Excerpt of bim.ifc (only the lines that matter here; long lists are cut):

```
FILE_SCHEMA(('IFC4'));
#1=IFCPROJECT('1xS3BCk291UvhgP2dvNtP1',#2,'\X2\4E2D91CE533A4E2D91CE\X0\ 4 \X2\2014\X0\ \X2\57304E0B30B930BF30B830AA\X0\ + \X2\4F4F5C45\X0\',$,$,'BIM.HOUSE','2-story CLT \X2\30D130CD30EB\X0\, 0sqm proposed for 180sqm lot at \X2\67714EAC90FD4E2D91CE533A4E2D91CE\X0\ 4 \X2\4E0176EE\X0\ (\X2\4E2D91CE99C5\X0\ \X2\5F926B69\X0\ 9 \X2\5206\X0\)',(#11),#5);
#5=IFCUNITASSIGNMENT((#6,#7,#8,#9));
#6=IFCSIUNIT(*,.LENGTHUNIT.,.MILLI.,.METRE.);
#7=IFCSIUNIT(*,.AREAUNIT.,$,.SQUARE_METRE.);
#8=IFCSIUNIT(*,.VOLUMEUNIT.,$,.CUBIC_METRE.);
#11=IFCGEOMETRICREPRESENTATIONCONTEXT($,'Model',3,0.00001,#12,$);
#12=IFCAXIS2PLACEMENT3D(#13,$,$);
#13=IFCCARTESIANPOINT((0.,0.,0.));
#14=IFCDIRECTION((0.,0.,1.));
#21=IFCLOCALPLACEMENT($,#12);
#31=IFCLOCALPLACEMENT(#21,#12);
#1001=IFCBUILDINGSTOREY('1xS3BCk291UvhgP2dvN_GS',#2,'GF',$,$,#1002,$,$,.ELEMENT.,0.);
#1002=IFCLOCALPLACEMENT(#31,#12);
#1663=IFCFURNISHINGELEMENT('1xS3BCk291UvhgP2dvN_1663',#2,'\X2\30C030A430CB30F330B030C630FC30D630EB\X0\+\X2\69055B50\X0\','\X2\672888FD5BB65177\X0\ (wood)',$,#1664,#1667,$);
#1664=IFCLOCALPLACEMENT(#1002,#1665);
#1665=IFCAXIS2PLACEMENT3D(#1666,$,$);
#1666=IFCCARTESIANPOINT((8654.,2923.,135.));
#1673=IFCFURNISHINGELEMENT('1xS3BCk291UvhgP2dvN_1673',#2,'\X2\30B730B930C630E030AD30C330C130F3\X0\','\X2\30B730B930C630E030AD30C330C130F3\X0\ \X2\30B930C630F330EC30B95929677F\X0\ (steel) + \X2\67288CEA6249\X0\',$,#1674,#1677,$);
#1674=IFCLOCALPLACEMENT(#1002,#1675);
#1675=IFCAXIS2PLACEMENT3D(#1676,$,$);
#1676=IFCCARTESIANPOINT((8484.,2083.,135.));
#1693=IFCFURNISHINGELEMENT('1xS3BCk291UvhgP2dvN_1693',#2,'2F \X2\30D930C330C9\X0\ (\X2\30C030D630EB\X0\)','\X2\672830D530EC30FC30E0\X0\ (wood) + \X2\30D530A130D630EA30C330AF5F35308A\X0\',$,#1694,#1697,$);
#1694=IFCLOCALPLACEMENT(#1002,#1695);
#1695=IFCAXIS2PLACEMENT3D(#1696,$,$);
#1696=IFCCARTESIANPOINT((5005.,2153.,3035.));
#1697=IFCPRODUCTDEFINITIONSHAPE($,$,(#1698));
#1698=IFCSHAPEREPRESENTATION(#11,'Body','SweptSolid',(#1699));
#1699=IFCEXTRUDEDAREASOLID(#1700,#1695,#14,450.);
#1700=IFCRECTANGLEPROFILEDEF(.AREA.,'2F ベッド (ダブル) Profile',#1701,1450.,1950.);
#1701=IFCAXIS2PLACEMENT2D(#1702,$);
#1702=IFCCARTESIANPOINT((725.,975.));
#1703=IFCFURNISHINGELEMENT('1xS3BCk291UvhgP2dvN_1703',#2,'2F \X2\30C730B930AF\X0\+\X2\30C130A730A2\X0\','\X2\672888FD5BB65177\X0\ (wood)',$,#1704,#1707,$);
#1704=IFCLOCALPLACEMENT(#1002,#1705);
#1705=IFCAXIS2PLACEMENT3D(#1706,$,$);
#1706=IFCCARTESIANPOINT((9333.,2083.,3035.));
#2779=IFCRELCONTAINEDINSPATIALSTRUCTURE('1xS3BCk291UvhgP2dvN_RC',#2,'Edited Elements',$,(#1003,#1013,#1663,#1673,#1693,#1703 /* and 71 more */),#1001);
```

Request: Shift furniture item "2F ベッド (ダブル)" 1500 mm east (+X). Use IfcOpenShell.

```python
import ifcopenshell
import ifcopenshell.api.geometry
import ifcopenshell.util.placement
import ifcopenshell.util.unit

model = ifcopenshell.open("bim.ifc")
unit_scale = ifcopenshell.util.unit.calculate_unit_scale(model)

item = model.by_guid("1xS3BCk291UvhgP2dvN_1693")
matrix = ifcopenshell.util.placement.get_local_placement(item.ObjectPlacement)
matrix[0, 3] += 1.5 / unit_scale
ifcopenshell.api.geometry.edit_object_placement(model, product=item, matrix=matrix, is_si=False)

print(ifcopenshell.util.placement.get_local_placement(item.ObjectPlacement).round(3) + 0.0)

model.write("bim_rev.ifc")
```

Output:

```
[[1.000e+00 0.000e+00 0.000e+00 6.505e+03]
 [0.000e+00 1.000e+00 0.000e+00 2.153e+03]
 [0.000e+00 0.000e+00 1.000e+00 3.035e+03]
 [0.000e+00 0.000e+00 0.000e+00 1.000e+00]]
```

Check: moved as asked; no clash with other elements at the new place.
